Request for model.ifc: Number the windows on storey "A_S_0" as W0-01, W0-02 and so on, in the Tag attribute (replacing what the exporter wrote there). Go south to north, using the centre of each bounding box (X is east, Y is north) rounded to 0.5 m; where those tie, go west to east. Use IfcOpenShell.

First a look at what the model holds.

```python
import ifcopenshell
import ifcopenshell.util.element
import ifcopenshell.util.placement

model = ifcopenshell.open("model.ifc")
print(model.schema)
storey = next(s for s in model.by_type("IfcBuildingStorey") if s.Name == "A_S_0")
windows = [e for e in ifcopenshell.util.element.get_decomposition(storey) if e.is_a("IfcWindow")]
for e in sorted(windows, key=lambda e: e.id()):
    origin = ifcopenshell.util.placement.get_local_placement(e.ObjectPlacement)[:3, 3]
    print(e.id(), e.Tag, e.Name, origin.round(2) + 0.0, sep=" | ")
```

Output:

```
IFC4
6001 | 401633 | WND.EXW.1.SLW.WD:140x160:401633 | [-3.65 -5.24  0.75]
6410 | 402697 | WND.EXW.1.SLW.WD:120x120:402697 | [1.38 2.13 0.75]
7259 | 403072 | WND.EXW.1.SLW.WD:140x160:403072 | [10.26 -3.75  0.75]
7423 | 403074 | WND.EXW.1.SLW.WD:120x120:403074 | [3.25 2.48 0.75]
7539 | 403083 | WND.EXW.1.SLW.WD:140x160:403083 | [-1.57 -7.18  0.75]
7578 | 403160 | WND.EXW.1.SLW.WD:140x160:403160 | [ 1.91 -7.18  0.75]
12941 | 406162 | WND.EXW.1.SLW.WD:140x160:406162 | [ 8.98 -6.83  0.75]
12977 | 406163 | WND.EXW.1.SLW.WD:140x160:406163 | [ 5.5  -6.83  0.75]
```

```python
import ifcopenshell
import ifcopenshell.geom
import ifcopenshell.util.element
import ifcopenshell.util.shape

model = ifcopenshell.open("model.ifc")
settings = ifcopenshell.geom.settings()
settings.set("use-world-coords", True)


def centre(element):
    shape = ifcopenshell.geom.create_shape(settings, element)
    return ifcopenshell.util.shape.get_bbox_centroid(shape.geometry)


storey = next(s for s in model.by_type("IfcBuildingStorey") if s.Name == "A_S_0")
windows = [e for e in ifcopenshell.util.element.get_decomposition(storey) if e.is_a("IfcWindow")]

# Insertion points can sit at a corner or the storey origin, so sort by the geometry (in metres).
centres = {e: centre(e) for e in windows}
windows.sort(key=lambda e: (round(centres[e][1] / 0.5), centres[e][0]))

for i, e in enumerate(windows, start=1):
    number = f"W0-{i:02d}"
    e.Tag = number
    print(e.id(), number)

model.write("model_rev.ifc")
```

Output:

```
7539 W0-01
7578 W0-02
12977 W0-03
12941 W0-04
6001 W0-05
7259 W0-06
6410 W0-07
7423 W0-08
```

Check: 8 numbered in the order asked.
